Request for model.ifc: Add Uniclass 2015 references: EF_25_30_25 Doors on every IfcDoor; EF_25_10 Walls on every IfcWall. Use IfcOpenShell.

First a look at what the model holds.

```python
import ifcopenshell

model = ifcopenshell.open("model.ifc")
print(model.schema)
print("classifications:", [c.Name for c in model.by_type("IfcClassification")])
for ifc_class in ("IfcDoor", "IfcRoof", "IfcStair", "IfcWall", "IfcWindow"):
    print(ifc_class, len(model.by_type(ifc_class)))
```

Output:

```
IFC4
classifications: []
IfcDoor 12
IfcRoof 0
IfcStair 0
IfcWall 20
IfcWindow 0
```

```python
import ifcopenshell
import ifcopenshell.api.classification

model = ifcopenshell.open("model.ifc")

system = ifcopenshell.api.classification.add_classification(model, classification="Uniclass 2015")

codes = {
    "IfcDoor": ("EF_25_30_25", "Doors"),
    "IfcWall": ("EF_25_10", "Walls"),
}
for ifc_class, (code, name) in codes.items():
    products = model.by_type(ifc_class)
    ifcopenshell.api.classification.add_reference(
        model, products=products, classification=system, identification=code, name=name
    )
    print(code, len(products))

model.write("model_edited.ifc")
```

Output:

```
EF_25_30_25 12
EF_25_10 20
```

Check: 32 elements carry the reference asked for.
